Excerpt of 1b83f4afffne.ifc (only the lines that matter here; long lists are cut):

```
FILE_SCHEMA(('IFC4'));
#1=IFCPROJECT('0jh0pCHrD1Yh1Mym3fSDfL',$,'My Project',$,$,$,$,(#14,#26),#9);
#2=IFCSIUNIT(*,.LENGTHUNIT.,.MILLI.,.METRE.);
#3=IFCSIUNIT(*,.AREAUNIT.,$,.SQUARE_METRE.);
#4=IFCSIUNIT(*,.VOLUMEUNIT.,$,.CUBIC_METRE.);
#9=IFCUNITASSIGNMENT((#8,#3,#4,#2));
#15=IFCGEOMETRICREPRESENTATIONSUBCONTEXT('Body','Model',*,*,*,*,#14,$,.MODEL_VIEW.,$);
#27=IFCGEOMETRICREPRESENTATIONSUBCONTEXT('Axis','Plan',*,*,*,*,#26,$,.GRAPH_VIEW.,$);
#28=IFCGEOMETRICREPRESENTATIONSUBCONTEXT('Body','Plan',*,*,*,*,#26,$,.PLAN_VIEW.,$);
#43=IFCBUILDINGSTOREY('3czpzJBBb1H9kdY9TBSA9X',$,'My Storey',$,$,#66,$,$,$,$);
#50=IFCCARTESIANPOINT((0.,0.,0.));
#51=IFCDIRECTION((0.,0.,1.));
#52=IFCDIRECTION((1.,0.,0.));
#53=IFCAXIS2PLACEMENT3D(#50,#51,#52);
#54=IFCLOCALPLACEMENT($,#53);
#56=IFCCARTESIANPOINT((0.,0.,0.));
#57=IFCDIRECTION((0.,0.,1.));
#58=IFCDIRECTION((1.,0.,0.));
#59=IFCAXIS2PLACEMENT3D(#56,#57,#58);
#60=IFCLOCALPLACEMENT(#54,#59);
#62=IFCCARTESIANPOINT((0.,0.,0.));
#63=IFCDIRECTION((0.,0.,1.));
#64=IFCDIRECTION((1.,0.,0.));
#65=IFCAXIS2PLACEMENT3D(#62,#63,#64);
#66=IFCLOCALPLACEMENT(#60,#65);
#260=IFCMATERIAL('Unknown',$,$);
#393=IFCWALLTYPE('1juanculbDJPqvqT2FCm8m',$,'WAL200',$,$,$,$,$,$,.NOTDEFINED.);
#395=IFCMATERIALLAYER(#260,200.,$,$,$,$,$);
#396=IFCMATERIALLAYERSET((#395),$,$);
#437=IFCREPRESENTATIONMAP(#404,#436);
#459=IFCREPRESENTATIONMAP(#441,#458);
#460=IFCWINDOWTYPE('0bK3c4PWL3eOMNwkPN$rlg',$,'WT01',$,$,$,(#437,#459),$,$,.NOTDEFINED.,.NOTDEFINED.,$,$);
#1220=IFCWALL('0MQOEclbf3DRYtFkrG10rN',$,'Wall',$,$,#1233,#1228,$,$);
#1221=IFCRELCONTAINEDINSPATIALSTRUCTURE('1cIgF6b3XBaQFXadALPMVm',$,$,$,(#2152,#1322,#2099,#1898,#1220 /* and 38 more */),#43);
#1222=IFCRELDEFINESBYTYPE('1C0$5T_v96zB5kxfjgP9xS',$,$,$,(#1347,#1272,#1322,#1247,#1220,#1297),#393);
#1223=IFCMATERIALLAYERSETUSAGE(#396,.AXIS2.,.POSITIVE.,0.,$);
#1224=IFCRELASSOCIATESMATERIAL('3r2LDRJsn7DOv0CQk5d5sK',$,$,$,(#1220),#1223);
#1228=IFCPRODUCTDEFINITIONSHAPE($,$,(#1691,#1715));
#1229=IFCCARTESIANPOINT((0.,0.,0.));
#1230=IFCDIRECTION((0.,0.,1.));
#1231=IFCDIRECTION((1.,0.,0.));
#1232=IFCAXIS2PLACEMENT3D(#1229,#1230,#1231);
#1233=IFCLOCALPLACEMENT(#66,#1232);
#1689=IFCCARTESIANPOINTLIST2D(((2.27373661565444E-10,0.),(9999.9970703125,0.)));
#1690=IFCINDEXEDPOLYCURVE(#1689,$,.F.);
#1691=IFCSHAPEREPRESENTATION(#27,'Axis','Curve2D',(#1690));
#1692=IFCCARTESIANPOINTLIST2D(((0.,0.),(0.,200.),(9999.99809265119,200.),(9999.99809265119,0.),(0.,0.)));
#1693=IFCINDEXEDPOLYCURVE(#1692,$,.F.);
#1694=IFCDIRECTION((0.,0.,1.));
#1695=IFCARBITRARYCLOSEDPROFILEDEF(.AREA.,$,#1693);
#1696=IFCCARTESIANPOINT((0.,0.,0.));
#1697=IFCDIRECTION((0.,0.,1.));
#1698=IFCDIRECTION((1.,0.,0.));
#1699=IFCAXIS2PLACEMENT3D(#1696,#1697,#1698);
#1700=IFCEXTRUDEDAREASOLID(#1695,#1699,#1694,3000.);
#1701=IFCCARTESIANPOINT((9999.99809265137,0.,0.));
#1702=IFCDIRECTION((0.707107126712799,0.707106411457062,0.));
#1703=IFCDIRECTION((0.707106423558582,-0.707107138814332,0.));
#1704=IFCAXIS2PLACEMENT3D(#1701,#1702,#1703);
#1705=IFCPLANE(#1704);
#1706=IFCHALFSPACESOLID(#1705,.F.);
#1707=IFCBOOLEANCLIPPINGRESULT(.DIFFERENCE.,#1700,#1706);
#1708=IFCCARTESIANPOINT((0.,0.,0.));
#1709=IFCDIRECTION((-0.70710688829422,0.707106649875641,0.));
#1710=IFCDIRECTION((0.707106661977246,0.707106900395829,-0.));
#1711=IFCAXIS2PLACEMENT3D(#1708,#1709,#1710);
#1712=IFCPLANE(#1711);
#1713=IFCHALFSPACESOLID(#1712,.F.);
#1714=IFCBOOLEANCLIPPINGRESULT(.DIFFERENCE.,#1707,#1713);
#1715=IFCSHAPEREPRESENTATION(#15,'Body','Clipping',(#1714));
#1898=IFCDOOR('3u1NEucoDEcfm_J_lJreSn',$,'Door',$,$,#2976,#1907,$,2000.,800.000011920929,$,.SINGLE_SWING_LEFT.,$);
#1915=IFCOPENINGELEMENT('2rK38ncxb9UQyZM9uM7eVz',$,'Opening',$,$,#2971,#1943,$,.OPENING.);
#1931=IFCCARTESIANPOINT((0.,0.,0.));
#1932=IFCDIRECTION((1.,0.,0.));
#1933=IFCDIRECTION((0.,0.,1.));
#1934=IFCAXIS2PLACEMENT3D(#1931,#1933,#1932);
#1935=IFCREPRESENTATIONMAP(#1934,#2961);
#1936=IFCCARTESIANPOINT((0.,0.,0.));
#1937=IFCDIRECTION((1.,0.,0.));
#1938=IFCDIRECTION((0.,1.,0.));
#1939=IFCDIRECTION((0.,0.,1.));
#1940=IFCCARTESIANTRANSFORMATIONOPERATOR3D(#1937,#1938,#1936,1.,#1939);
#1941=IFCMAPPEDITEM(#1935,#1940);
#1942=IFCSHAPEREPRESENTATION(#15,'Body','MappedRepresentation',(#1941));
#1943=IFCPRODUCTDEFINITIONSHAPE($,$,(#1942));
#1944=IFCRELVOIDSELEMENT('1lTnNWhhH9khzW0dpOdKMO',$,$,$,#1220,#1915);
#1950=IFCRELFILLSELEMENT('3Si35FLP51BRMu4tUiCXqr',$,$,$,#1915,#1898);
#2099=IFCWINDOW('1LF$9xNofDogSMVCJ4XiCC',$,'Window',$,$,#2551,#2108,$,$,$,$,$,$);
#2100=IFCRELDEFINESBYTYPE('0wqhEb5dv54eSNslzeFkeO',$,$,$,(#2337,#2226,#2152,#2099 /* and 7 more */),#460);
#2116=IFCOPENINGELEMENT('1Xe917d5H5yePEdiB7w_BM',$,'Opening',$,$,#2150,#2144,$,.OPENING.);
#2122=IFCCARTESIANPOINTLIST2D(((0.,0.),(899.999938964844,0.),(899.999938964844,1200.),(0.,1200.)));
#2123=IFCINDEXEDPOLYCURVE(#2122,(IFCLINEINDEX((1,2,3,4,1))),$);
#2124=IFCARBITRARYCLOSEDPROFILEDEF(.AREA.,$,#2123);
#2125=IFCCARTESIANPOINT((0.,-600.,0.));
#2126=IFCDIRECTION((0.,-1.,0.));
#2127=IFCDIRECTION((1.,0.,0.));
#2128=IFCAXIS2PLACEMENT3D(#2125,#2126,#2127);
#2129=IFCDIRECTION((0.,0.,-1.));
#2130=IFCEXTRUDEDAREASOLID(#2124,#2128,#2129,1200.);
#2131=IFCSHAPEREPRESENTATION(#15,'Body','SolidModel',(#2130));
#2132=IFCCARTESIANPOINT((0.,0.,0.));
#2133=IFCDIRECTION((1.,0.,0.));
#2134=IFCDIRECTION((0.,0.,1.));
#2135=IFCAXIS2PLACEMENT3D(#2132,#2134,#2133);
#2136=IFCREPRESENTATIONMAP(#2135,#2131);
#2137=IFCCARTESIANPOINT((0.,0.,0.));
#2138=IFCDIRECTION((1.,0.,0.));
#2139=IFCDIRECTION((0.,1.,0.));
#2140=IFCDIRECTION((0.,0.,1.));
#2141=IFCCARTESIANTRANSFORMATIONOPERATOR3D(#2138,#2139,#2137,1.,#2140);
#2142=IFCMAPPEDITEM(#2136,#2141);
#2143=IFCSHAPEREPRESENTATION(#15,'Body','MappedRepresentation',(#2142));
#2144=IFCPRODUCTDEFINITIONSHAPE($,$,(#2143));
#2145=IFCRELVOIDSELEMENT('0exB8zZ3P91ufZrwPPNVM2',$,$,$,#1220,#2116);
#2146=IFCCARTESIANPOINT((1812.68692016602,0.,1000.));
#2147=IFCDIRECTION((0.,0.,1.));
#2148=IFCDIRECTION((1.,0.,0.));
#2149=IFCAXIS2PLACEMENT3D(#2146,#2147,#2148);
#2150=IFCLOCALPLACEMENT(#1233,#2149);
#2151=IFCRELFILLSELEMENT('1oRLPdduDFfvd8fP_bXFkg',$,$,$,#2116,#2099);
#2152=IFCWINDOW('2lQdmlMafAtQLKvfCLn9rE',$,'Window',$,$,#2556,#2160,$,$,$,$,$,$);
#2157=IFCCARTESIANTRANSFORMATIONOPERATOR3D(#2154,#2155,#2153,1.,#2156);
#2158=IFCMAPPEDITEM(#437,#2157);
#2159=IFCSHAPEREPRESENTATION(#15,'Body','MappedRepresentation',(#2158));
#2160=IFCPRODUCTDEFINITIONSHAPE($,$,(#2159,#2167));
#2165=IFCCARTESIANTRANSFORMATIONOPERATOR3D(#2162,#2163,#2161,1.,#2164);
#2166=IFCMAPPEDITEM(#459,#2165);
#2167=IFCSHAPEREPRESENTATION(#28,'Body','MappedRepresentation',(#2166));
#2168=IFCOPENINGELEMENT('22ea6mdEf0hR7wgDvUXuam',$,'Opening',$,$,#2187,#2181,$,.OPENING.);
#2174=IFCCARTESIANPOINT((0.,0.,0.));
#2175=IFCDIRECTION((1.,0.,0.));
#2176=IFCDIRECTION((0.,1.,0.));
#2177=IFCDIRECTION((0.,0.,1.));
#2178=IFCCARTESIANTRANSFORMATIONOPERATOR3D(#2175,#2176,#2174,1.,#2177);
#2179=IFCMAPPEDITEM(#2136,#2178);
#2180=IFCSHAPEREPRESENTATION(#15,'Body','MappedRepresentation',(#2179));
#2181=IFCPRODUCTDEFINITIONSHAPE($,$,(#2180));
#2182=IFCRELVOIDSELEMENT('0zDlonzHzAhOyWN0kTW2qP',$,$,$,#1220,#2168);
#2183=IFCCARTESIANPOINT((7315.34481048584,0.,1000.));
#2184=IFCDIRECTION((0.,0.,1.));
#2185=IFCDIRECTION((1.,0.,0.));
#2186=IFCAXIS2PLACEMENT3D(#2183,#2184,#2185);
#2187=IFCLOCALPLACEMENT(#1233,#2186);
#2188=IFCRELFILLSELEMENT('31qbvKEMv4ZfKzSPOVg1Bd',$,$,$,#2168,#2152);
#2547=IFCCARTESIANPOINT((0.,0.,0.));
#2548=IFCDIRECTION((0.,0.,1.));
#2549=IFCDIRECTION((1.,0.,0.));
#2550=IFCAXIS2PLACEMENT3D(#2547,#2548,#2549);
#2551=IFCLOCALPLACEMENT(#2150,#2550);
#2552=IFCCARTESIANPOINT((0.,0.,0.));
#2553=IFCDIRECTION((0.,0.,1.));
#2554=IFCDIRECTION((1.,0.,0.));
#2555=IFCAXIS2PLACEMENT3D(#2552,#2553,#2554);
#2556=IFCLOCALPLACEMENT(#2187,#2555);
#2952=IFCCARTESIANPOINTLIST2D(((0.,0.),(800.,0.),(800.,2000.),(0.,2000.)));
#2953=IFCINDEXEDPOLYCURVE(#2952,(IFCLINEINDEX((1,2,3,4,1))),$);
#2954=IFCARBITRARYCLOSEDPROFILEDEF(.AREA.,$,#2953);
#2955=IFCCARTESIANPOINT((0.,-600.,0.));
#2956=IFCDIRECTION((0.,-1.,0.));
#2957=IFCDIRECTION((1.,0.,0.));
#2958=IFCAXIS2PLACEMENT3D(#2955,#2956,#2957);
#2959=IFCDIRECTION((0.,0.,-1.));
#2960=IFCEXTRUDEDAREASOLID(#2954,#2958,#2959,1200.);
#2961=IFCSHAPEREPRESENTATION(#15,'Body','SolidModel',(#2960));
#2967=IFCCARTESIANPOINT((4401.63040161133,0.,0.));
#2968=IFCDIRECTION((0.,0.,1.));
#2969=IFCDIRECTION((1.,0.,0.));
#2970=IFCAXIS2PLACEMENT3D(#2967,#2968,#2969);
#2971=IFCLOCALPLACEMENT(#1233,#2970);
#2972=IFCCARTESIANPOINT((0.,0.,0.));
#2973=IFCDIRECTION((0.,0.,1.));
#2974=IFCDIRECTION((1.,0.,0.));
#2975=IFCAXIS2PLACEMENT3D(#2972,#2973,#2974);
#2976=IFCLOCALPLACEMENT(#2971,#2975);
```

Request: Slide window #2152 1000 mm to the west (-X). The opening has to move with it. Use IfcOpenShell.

```python
import ifcopenshell
import ifcopenshell.api.geometry
import ifcopenshell.util.placement
import ifcopenshell.util.unit

model = ifcopenshell.open("1b83f4afffne.ifc")
unit_scale = ifcopenshell.util.unit.calculate_unit_scale(model)

window = model.by_id(2152)
opening = window.FillsVoids[0].RelatingOpeningElement
wall = opening.VoidsElements[0].RelatingBuildingElement

wall_matrix = ifcopenshell.util.placement.get_local_placement(wall.ObjectPlacement)
shift = wall_matrix[:3, 0] * -1 / unit_scale
before = ifcopenshell.util.placement.get_local_placement(window.ObjectPlacement)[:3, 3].copy()

# The window is placed relative to its opening, so it follows when the opening moves.
matrix = ifcopenshell.util.placement.get_local_placement(opening.ObjectPlacement)
matrix[:3, 3] += shift
ifcopenshell.api.geometry.edit_object_placement(
    model, product=opening, matrix=matrix, is_si=False, should_transform_children=True
)

after = ifcopenshell.util.placement.get_local_placement(window.ObjectPlacement)[:3, 3]
print("window moved by", (after - before).round(3) + 0.0)

model.write("1b83f4afffne_rev.ifc")
```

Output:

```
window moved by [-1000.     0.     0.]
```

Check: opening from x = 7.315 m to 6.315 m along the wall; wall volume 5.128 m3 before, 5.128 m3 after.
